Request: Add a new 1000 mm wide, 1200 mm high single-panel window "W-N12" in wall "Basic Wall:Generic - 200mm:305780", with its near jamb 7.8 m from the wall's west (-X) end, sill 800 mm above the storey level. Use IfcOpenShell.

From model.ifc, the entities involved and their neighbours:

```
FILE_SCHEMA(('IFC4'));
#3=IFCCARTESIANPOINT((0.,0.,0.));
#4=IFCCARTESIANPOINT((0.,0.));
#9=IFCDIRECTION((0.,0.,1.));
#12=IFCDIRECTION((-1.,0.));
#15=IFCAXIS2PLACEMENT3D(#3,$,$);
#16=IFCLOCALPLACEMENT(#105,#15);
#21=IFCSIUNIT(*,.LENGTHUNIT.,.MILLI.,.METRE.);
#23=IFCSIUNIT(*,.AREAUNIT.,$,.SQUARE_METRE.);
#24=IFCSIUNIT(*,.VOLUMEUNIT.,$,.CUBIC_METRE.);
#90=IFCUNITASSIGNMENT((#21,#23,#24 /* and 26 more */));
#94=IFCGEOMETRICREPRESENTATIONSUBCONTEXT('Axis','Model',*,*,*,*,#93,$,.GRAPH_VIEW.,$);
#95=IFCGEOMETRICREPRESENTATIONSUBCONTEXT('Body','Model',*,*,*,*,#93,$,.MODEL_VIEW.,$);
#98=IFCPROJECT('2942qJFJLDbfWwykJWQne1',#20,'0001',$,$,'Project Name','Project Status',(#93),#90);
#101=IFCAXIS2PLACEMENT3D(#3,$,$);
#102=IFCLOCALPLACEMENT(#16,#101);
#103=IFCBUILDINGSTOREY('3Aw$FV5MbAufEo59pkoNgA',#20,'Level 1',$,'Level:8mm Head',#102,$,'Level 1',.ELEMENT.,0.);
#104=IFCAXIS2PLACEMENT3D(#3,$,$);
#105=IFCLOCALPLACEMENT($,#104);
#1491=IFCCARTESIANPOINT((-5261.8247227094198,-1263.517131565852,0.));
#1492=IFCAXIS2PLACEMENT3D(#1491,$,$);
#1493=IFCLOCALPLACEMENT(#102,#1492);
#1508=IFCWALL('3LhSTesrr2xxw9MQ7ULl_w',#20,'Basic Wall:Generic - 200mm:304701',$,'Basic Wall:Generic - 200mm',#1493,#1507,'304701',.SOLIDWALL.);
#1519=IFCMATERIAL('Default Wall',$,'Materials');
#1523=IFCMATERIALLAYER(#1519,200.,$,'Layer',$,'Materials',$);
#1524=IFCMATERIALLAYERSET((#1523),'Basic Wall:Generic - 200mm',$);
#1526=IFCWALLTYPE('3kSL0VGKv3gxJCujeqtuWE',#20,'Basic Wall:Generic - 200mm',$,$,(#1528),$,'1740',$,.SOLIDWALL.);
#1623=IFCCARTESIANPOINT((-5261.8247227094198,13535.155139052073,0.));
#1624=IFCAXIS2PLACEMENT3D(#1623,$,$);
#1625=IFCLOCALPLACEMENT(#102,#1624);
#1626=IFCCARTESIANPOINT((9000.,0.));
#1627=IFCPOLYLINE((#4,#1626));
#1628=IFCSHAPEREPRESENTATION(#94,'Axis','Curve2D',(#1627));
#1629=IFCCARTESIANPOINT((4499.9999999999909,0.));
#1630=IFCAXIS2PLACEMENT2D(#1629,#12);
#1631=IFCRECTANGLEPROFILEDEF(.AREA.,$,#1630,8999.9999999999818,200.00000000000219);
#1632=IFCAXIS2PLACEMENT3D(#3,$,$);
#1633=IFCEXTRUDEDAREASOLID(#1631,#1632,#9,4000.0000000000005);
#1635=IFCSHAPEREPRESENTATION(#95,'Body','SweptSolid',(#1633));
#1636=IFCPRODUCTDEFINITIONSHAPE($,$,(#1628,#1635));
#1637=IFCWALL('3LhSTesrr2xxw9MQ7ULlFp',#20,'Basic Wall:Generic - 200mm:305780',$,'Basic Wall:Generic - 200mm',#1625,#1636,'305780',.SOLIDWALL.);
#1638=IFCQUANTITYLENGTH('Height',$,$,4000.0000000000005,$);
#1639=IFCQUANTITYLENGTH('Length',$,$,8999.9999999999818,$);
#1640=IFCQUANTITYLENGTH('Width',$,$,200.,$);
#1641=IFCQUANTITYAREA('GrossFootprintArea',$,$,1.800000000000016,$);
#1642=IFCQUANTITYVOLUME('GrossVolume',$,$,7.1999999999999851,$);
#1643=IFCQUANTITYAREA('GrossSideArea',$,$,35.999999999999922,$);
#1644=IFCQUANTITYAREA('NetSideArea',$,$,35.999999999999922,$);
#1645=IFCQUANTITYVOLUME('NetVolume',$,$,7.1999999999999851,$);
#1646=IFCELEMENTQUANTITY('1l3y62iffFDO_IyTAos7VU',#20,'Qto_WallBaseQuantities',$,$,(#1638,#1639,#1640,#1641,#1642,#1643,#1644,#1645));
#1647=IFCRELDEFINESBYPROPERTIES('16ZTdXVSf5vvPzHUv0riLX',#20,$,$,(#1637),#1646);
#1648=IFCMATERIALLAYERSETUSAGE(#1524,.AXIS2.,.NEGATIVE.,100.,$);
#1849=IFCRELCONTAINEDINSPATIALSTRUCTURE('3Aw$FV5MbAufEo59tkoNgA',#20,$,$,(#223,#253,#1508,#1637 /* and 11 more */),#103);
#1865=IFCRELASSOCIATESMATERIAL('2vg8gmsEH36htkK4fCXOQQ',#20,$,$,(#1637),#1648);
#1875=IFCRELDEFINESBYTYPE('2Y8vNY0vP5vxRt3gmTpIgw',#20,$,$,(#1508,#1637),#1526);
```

```python
import numpy as np
import ifcopenshell
import ifcopenshell.api.feature
import ifcopenshell.api.geometry
import ifcopenshell.api.pset
import ifcopenshell.api.root
import ifcopenshell.api.spatial
import ifcopenshell.geom
import ifcopenshell.util.element
import ifcopenshell.util.placement
import ifcopenshell.util.representation
import ifcopenshell.util.shape
import ifcopenshell.util.unit

model = ifcopenshell.open("model.ifc")
unit_scale = ifcopenshell.util.unit.calculate_unit_scale(model)
area_scale = ifcopenshell.util.unit.calculate_unit_scale(model, "AREAUNIT")
volume_scale = ifcopenshell.util.unit.calculate_unit_scale(model, "VOLUMEUNIT")
settings = ifcopenshell.geom.settings()


def volume(element):
    """Net volume in cubic metres, openings subtracted."""
    shape = ifcopenshell.geom.create_shape(settings, element)
    return ifcopenshell.util.shape.get_volume(shape.geometry)


wall = model.by_id(1637)
storey = ifcopenshell.util.element.get_container(wall, ifc_class="IfcBuildingStorey")
context = ifcopenshell.util.representation.get_context(model, "Model", "Body", "MODEL_VIEW")
before = volume(wall)

width, height, from_end, sill = 1, 1.2, 7.8, 0.8  # metres

# The wall runs along its own X axis, and the end named is its -X end.
wall_shape = ifcopenshell.geom.create_shape(settings, wall)
x, y, z = ifcopenshell.util.shape.get_vertices(wall_shape.geometry).T
start = x.min() + from_end
face, thickness = float(y.min()), float(y.max() - y.min())
wall_matrix = ifcopenshell.util.placement.get_local_placement(wall.ObjectPlacement)
level = ifcopenshell.util.placement.get_local_placement(storey.ObjectPlacement)[2, 3]


def in_wall(x, y):
    """Placement at x, y metres in the wall's axes, at sill height."""
    matrix = wall_matrix.copy()
    matrix[:, 3] = wall_matrix @ np.array([x / unit_scale, y / unit_scale, 0.0, 1.0])
    matrix[2, 3] = level + sill / unit_scale
    return matrix


# Opening: a box that overshoots both wall faces by 50 mm.
opening = ifcopenshell.api.root.create_entity(model, ifc_class="IfcOpeningElement", predefined_type="OPENING")
box = ifcopenshell.api.geometry.add_wall_representation(
    model, context=context, length=width, height=height, thickness=thickness + 0.1
)
ifcopenshell.api.geometry.assign_representation(model, product=opening, representation=box)
ifcopenshell.api.geometry.edit_object_placement(model, product=opening, matrix=in_wall(start, face - 0.05), is_si=False)
ifcopenshell.api.feature.add_feature(model, feature=opening, element=wall)

window = ifcopenshell.api.root.create_entity(model, ifc_class="IfcWindow", name="W-N12", predefined_type="WINDOW")
window.OverallWidth, window.OverallHeight = width / unit_scale, height / unit_scale
window.PartitioningType = "SINGLE_PANEL"
body = ifcopenshell.api.geometry.add_window_representation(
    model,
    context=context,
    overall_width=window.OverallWidth,
    overall_height=window.OverallHeight,
    partition_type="SINGLE_PANEL",
)
ifcopenshell.api.geometry.assign_representation(model, product=window, representation=body)
ifcopenshell.api.spatial.assign_container(model, products=[window], relating_structure=storey)
ifcopenshell.api.feature.add_filling(model, opening=opening, element=window)

# Centre the window in the wall's thickness.
ifcopenshell.api.geometry.edit_object_placement(model, product=window, matrix=in_wall(start, face), is_si=False)
window_shape = ifcopenshell.geom.create_shape(settings, window)
depth = ifcopenshell.util.shape.get_vertices(window_shape.geometry)[:, 1]
offset = face + thickness / 2 - (depth.min() + depth.max()) / 2
ifcopenshell.api.geometry.edit_object_placement(model, product=window, matrix=in_wall(start, offset), is_si=False)

after = volume(wall)

# Update the wall's stored quantities.
qto = model.by_id(ifcopenshell.util.element.get_pset(wall, "Qto_WallBaseQuantities", should_inherit=False)["id"])
ifcopenshell.api.pset.edit_qto(model, qto=qto, properties={
    "NetSideArea": after / thickness / area_scale,
    "NetVolume": after / volume_scale,
})

print(f"wall volume {before:.3f} -> {after:.3f} m3")

model.write("model_edited.ifc")
```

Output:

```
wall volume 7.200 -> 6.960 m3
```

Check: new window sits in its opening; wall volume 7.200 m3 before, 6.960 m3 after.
